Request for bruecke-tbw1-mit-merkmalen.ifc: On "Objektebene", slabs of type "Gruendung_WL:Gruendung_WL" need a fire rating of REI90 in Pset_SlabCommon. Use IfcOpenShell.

First a look at what the model holds.

```python
import ifcopenshell
import ifcopenshell.util.element

model = ifcopenshell.open("bruecke-tbw1-mit-merkmalen.ifc")
print(model.schema)
storey = next(s for s in model.by_type("IfcBuildingStorey") if s.Name == "Objektebene")
slabs = [e for e in ifcopenshell.util.element.get_decomposition(storey) if e.is_a("IfcSlab")]
seen = {}
for e in slabs:
    element_type = ifcopenshell.util.element.get_type(e)
    key = (element_type.Name if element_type != e and element_type else None, ifcopenshell.util.element.get_pset(e, "Pset_SlabCommon", "FireRating"))
    seen[key] = seen.get(key, 0) + 1
for (name, value), count in sorted(seen.items(), key=str):
    print(count, "x", name, "|", value)
```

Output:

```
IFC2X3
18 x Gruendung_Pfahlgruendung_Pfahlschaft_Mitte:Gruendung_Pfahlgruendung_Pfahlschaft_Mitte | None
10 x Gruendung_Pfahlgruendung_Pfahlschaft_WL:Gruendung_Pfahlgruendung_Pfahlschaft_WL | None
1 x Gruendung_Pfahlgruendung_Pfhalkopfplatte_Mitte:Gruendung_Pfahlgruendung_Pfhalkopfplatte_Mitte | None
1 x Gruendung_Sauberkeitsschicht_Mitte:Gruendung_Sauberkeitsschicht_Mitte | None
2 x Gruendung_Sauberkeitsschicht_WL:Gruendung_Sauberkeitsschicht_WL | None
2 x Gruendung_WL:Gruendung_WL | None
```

```python
import ifcopenshell
import ifcopenshell.api.pset
import ifcopenshell.util.element

model = ifcopenshell.open("bruecke-tbw1-mit-merkmalen.ifc")

storey = next(s for s in model.by_type("IfcBuildingStorey") if s.Name == "Objektebene")
slabs = [e for e in ifcopenshell.util.element.get_decomposition(storey) if e.is_a("IfcSlab")]

count = 0
for e in slabs:
    element_type = ifcopenshell.util.element.get_type(e)
    if element_type in (None, e) or element_type.Name != "Gruendung_WL:Gruendung_WL":
        continue
    # add_pset returns the element's existing set when there is one.
    pset = ifcopenshell.api.pset.add_pset(model, product=e, name="Pset_SlabCommon")
    ifcopenshell.api.pset.edit_pset(model, pset=pset, properties={"FireRating": "REI90"})
    count += 1

print(count, "slabs updated")

model.write("bruecke-tbw1-mit-merkmalen_edited.ifc")
```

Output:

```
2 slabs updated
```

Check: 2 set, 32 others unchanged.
